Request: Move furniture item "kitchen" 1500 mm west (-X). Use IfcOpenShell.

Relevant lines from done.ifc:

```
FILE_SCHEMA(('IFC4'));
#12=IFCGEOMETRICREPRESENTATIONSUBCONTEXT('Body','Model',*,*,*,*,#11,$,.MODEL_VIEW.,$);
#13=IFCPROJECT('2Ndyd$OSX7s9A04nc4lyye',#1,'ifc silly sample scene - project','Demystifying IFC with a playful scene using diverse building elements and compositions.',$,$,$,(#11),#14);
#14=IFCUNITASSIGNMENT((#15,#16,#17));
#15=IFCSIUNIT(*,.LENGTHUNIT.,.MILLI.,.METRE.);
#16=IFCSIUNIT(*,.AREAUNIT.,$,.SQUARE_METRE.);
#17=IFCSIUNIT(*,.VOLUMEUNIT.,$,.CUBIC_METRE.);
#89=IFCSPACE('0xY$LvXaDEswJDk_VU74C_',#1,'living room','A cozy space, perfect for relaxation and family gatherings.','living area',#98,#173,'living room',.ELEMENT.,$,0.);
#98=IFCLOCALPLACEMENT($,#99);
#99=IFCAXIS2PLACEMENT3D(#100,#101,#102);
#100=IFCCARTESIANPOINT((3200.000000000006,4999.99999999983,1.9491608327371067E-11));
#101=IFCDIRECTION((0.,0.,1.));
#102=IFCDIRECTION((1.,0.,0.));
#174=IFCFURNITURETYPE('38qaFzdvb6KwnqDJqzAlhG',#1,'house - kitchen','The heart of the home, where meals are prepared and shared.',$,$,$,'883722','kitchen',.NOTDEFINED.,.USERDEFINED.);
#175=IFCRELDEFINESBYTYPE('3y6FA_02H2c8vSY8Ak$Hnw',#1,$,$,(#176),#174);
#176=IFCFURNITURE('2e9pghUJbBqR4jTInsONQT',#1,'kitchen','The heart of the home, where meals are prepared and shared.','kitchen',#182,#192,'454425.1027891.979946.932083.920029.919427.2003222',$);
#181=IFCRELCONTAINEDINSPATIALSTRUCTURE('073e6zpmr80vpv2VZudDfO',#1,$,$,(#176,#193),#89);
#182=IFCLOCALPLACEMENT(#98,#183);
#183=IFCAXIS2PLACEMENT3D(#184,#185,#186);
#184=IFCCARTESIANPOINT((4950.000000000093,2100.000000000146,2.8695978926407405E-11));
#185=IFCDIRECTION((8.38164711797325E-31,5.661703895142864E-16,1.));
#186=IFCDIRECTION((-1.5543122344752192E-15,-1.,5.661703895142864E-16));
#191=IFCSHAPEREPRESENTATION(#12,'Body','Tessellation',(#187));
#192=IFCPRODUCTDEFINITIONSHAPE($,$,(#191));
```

```python
import ifcopenshell
import ifcopenshell.api.geometry
import ifcopenshell.util.placement
import ifcopenshell.util.unit

model = ifcopenshell.open("done.ifc")
unit_scale = ifcopenshell.util.unit.calculate_unit_scale(model)

item = model.by_guid("2e9pghUJbBqR4jTInsONQT")
matrix = ifcopenshell.util.placement.get_local_placement(item.ObjectPlacement)
matrix[0, 3] -= 1.5 / unit_scale
ifcopenshell.api.geometry.edit_object_placement(model, product=item, matrix=matrix, is_si=False)

print(ifcopenshell.util.placement.get_local_placement(item.ObjectPlacement).round(3) + 0.0)

model.write("done_edited.ifc")
```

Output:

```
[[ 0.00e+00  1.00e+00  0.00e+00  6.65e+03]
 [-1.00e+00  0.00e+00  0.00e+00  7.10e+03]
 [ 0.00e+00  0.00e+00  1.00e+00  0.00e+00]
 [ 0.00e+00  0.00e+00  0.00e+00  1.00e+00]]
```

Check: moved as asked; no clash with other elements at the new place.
